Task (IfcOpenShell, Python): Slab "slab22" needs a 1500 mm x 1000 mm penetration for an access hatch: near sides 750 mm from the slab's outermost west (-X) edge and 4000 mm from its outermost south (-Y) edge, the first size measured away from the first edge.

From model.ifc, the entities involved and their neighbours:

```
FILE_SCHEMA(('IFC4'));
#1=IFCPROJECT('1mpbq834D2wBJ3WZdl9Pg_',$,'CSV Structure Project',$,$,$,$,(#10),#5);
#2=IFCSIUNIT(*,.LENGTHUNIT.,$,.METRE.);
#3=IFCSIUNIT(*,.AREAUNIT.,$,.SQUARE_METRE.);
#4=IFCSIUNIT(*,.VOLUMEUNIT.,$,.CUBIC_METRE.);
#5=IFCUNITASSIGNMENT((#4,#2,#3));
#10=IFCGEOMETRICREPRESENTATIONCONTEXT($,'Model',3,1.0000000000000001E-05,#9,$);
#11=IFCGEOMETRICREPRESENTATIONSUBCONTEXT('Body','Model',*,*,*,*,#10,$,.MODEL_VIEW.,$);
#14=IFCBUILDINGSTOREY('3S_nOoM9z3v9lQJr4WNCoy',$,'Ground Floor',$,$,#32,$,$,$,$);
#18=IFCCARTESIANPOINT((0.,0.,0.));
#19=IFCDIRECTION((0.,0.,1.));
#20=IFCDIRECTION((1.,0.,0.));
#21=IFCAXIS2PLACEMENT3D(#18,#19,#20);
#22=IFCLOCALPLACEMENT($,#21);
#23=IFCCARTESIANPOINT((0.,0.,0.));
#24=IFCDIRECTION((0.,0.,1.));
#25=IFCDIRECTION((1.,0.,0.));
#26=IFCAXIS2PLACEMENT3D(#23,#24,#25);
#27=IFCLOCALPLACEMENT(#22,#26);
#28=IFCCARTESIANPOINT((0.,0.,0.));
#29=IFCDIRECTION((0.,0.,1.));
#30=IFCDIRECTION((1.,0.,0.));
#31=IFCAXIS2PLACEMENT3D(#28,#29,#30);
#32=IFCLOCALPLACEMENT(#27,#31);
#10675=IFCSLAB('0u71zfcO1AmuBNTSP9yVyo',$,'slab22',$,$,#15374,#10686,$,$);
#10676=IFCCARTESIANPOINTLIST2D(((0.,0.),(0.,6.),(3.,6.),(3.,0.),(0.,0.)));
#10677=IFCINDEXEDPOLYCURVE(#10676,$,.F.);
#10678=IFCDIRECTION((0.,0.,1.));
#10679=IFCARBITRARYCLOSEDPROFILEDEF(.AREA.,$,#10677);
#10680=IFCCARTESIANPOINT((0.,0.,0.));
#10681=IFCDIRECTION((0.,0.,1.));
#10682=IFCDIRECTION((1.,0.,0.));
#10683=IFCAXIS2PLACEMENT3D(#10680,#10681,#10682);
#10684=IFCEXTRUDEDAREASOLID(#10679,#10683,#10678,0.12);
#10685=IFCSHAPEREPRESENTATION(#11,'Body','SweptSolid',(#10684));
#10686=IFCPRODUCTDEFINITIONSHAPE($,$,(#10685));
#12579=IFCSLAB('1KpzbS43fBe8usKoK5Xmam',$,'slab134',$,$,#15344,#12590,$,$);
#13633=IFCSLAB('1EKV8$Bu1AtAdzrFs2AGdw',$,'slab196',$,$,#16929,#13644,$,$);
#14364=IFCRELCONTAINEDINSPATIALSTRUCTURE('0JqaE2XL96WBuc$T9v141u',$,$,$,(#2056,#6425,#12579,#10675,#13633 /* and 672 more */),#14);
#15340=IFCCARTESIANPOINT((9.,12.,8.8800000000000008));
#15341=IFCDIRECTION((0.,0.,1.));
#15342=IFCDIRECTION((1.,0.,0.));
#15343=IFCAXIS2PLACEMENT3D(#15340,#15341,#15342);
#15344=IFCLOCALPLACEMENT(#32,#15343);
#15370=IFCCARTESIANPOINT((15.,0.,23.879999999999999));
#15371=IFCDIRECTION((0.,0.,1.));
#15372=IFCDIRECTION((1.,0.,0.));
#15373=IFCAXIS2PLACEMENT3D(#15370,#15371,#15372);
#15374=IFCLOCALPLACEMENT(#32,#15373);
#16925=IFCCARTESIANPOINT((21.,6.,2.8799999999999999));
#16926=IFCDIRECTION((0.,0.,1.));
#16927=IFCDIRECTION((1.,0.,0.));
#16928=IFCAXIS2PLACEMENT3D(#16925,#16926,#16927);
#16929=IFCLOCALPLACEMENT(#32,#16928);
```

```python
import numpy as np
import ifcopenshell
import ifcopenshell.api.feature
import ifcopenshell.api.geometry
import ifcopenshell.api.root
import ifcopenshell.geom
import ifcopenshell.util.placement
import ifcopenshell.util.representation
import ifcopenshell.util.shape
import ifcopenshell.util.unit

model = ifcopenshell.open("model.ifc")
unit_scale = ifcopenshell.util.unit.calculate_unit_scale(model)
settings = ifcopenshell.geom.settings()


def volume(element):
    """Net volume in cubic metres, openings subtracted."""
    shape = ifcopenshell.geom.create_shape(settings, element)
    return ifcopenshell.util.shape.get_volume(shape.geometry)


slab = model.by_id(10675)
before = volume(slab)

# Extent in the slab's own axes, in metres. The edges named are its -X and -Y sides.
slab_shape = ifcopenshell.geom.create_shape(settings, slab)
vertices = ifcopenshell.util.shape.get_vertices(slab_shape.geometry)
x_min, y_min, bottom = vertices.min(axis=0)
top = vertices[:, 2].max()

opening = ifcopenshell.api.root.create_entity(model, ifc_class="IfcOpeningElement", name="Access hatch opening", predefined_type="OPENING")
context = ifcopenshell.util.representation.get_context(model, "Model", "Body", "MODEL_VIEW")
width, depth = 1.5, 1
outline = [(0.0, 0.0), (width, 0.0), (width, depth), (0.0, depth), (0.0, 0.0)]
# Overshoot both faces by 50 mm so the cut is clean.
shape = ifcopenshell.api.geometry.add_slab_representation(
    model, context=context, depth=top - bottom + 0.1, polyline=outline
)
ifcopenshell.api.geometry.assign_representation(model, product=opening, representation=shape)

matrix = ifcopenshell.util.placement.get_local_placement(slab.ObjectPlacement)
matrix[:, 3] = matrix @ np.append(np.array([x_min + 0.75, y_min + 4, bottom - 0.05]) / unit_scale, 1.0)
ifcopenshell.api.geometry.edit_object_placement(model, product=opening, matrix=matrix, is_si=False)
ifcopenshell.api.feature.add_feature(model, feature=opening, element=slab)

after = volume(slab)

print(f"slab volume {before:.3f} -> {after:.3f} m3")

model.write("model-out.ifc")
```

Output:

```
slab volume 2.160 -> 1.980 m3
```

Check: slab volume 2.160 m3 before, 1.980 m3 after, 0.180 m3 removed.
